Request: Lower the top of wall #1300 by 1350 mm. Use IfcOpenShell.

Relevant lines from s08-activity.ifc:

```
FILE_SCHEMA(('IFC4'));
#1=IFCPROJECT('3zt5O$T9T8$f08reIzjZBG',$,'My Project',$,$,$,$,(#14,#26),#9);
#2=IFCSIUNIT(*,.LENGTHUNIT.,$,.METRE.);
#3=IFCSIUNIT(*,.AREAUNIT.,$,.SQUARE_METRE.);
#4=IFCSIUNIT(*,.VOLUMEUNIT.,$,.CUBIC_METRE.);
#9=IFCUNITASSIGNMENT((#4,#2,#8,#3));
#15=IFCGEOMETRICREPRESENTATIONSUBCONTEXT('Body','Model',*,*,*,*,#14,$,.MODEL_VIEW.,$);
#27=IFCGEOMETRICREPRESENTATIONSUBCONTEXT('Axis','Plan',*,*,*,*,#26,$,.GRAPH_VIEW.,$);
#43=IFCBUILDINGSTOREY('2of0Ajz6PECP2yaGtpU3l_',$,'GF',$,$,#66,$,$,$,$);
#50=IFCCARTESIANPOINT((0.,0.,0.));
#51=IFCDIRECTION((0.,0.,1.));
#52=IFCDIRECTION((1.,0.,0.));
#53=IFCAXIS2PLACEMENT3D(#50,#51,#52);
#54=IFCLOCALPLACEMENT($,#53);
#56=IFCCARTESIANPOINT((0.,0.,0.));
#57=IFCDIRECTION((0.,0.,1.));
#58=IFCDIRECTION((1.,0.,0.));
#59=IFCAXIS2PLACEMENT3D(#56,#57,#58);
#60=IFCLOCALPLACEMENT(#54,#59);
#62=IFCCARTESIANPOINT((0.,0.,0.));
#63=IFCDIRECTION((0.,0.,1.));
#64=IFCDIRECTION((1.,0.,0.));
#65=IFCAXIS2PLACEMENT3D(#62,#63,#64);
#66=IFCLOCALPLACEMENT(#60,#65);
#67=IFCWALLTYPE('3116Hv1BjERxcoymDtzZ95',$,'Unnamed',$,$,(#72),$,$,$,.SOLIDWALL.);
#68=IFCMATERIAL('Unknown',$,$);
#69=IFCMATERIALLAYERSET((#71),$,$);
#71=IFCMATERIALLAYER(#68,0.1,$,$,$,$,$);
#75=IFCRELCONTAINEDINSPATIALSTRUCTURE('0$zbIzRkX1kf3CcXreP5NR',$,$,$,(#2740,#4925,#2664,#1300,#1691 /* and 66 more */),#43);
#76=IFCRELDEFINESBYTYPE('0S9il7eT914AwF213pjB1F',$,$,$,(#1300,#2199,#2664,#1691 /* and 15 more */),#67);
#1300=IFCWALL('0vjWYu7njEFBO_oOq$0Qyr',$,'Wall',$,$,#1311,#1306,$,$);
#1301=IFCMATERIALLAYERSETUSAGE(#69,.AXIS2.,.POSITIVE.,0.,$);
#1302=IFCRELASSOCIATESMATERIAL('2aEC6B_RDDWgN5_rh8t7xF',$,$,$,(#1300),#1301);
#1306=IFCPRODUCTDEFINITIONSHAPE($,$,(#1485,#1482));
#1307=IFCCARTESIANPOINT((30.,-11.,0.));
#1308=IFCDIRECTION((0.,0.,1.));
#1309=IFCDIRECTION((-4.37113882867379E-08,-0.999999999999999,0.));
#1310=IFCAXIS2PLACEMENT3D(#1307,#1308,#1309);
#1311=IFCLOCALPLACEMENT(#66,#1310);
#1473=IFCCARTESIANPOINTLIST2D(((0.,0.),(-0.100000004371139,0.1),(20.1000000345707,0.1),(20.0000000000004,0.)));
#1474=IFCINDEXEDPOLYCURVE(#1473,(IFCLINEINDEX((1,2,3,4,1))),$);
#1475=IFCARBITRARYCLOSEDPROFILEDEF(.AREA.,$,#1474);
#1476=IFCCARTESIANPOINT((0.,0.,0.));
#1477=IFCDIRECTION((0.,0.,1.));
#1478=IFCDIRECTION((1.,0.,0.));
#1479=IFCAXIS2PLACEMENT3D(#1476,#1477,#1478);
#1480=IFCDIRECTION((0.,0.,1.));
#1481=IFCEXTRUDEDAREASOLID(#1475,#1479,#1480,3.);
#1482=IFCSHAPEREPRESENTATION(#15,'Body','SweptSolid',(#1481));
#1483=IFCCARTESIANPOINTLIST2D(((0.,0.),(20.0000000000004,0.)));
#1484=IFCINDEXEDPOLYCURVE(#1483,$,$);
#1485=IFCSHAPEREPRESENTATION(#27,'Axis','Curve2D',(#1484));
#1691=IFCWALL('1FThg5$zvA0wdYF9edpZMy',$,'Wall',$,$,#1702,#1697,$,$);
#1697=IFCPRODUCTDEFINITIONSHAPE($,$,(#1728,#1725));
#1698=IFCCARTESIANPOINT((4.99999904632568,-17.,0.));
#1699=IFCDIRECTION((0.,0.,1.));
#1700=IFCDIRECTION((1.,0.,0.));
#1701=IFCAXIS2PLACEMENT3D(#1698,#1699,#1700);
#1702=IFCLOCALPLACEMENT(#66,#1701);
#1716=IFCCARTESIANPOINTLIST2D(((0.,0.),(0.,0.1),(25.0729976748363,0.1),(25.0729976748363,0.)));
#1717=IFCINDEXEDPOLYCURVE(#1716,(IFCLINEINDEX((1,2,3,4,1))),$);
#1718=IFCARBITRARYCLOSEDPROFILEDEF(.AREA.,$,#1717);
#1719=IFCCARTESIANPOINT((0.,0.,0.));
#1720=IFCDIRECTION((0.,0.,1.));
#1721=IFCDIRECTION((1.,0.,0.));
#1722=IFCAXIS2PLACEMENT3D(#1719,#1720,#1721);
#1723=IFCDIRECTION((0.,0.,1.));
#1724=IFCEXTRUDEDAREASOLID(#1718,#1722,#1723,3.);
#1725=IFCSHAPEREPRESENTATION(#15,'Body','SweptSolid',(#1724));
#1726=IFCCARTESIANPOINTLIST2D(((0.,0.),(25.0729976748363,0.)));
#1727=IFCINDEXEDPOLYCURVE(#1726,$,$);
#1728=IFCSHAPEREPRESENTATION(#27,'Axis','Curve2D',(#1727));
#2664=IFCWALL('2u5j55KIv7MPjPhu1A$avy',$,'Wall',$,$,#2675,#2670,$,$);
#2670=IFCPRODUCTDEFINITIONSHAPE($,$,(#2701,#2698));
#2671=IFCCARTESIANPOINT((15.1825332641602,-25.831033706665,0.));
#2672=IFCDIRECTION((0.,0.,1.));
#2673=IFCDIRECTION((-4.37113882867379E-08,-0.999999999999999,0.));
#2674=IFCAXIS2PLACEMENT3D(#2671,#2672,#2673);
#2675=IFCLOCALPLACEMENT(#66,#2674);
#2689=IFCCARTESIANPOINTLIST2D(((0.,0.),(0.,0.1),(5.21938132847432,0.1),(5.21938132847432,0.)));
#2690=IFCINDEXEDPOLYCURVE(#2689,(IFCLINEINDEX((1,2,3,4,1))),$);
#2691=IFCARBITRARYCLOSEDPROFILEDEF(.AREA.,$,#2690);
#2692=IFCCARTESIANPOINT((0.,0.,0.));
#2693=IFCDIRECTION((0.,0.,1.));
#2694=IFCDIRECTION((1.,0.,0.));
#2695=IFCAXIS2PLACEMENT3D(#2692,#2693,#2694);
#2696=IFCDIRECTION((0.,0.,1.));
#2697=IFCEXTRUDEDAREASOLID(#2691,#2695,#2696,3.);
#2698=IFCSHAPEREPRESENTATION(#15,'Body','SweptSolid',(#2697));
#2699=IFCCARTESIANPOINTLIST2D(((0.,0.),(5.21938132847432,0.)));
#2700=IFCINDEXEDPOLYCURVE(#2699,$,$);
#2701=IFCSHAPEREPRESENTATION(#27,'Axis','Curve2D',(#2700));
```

```python
import ifcopenshell
import ifcopenshell.geom
import ifcopenshell.util.representation
import ifcopenshell.util.shape

model = ifcopenshell.open("s08-activity.ifc")
settings = ifcopenshell.geom.settings()


def volume(element):
    """Net volume in cubic metres, openings subtracted."""
    shape = ifcopenshell.geom.create_shape(settings, element)
    return ifcopenshell.util.shape.get_volume(shape.geometry)


wall = model.by_id(1300)
before = volume(wall)

body = ifcopenshell.util.representation.get_representation(wall, "Model", "Body")
solid = body.Items[0]
old_height = solid.Depth
solid.Depth -= 1.35
after = volume(wall)

print(f"height {old_height:g} -> {solid.Depth:g}, volume {before:.3f} -> {after:.3f} m3")

model.write("s08-activity_edited.ifc")
```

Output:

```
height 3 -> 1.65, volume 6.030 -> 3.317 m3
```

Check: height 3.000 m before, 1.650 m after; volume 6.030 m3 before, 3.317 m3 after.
